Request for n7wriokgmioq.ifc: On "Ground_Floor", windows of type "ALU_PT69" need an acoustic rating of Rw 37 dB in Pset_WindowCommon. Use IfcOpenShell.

First a look at what the model holds.

```python
import ifcopenshell
import ifcopenshell.util.element

model = ifcopenshell.open("n7wriokgmioq.ifc")
print(model.schema)
storey = next(s for s in model.by_type("IfcBuildingStorey") if s.Name == "Ground_Floor")
windows = [e for e in ifcopenshell.util.element.get_decomposition(storey) if e.is_a("IfcWindow")]
seen = {}
for e in windows:
    element_type = ifcopenshell.util.element.get_type(e)
    key = (element_type.Name if element_type != e and element_type else None, ifcopenshell.util.element.get_pset(e, "Pset_WindowCommon", "AcousticRating"))
    seen[key] = seen.get(key, 0) + 1
for (name, value), count in sorted(seen.items(), key=str):
    print(count, "x", name, "|", value)
```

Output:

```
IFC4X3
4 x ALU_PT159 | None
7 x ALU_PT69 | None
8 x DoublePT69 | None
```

```python
import ifcopenshell
import ifcopenshell.api.pset
import ifcopenshell.util.element

model = ifcopenshell.open("n7wriokgmioq.ifc")

storey = next(s for s in model.by_type("IfcBuildingStorey") if s.Name == "Ground_Floor")
windows = [e for e in ifcopenshell.util.element.get_decomposition(storey) if e.is_a("IfcWindow")]

count = 0
for e in windows:
    element_type = ifcopenshell.util.element.get_type(e)
    if element_type in (None, e) or element_type.Name != "ALU_PT69":
        continue
    # add_pset returns the element's existing set when there is one.
    pset = ifcopenshell.api.pset.add_pset(model, product=e, name="Pset_WindowCommon")
    ifcopenshell.api.pset.edit_pset(model, pset=pset, properties={"AcousticRating": "Rw 37 dB"})
    count += 1

print(count, "windows updated")

model.write("n7wriokgmioq_rev.ifc")
```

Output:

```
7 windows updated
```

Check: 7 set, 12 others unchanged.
